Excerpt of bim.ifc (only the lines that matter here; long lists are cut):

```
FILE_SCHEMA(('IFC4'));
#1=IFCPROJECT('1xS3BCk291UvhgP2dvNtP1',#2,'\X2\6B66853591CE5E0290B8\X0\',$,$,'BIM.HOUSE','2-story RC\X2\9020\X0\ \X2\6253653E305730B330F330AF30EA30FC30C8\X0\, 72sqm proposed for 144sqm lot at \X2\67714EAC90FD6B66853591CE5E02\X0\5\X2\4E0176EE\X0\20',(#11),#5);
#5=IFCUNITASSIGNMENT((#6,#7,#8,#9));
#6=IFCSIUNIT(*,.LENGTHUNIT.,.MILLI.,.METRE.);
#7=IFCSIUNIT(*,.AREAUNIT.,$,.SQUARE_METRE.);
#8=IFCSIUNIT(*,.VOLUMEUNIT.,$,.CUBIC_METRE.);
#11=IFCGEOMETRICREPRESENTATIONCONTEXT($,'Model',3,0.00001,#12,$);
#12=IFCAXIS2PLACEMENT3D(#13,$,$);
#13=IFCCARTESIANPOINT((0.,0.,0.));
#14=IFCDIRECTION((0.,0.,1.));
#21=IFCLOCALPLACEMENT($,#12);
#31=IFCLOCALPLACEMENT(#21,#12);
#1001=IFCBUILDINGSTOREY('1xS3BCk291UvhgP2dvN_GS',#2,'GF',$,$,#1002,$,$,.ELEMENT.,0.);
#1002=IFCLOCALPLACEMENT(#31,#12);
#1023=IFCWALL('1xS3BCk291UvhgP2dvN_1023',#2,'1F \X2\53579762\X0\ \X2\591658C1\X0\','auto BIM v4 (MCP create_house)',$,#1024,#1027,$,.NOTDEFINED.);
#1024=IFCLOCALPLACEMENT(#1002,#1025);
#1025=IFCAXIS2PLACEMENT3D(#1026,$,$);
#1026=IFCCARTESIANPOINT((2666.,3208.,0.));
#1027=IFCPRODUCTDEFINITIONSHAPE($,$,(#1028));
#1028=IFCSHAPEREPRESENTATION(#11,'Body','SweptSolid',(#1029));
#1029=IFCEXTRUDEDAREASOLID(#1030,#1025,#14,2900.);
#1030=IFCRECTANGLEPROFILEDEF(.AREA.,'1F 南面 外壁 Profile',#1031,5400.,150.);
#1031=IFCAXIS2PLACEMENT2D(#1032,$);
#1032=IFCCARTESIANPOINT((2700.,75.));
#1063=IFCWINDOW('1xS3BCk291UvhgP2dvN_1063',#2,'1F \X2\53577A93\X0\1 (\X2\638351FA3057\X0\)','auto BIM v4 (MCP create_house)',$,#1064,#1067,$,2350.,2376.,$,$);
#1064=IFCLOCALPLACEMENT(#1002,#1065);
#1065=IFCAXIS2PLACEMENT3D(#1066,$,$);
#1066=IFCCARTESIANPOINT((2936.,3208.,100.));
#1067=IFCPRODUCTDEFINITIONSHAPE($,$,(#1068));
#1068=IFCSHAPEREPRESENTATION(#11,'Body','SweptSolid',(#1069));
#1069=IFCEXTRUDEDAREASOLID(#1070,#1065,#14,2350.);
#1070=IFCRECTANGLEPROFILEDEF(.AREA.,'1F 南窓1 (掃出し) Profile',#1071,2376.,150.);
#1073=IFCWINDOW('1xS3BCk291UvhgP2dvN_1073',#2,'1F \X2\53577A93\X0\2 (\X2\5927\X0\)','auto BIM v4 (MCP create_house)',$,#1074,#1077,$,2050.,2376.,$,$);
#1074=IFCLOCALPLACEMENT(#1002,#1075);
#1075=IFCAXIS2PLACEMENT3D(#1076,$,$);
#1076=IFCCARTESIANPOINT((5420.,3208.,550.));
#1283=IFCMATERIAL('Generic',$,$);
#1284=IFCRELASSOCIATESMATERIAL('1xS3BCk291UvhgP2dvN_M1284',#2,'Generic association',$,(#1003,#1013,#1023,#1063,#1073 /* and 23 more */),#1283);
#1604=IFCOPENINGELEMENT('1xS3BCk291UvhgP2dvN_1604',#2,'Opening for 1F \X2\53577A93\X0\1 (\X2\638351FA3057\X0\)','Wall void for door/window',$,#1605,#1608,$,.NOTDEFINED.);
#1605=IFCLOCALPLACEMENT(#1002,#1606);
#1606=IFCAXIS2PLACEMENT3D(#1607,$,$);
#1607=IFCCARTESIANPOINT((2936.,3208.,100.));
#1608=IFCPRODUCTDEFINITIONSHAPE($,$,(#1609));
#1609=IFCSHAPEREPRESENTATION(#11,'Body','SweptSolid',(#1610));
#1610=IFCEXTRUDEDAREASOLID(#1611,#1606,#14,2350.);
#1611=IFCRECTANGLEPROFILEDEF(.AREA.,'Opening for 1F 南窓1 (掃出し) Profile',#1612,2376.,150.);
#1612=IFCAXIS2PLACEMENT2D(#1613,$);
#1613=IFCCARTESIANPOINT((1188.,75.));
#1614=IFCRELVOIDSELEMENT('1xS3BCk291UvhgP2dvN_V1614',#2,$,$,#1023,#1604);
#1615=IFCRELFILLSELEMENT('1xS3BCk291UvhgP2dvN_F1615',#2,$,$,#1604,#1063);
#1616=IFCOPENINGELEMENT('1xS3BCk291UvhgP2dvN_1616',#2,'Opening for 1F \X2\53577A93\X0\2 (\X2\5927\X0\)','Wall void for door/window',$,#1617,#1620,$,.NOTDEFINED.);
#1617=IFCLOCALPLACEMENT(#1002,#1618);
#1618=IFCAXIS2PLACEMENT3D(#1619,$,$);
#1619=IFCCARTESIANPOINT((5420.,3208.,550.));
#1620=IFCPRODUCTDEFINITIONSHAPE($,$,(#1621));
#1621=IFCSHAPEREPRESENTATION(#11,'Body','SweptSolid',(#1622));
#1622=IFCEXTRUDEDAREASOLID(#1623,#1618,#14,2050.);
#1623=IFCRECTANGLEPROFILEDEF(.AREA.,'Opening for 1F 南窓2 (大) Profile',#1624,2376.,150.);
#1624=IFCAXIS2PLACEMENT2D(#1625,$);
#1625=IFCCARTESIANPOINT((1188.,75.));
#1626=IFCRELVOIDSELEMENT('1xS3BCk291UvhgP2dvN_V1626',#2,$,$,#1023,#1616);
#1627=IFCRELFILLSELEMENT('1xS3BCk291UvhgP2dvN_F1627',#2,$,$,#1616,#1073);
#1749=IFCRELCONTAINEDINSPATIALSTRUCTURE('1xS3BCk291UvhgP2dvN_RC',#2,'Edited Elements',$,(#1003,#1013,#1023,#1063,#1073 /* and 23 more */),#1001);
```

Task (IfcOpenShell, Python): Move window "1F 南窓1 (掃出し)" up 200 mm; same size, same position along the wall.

```python
import numpy as np
import ifcopenshell
import ifcopenshell.api.geometry
import ifcopenshell.util.placement
import ifcopenshell.util.unit

model = ifcopenshell.open("bim.ifc")
unit_scale = ifcopenshell.util.unit.calculate_unit_scale(model)

window = model.by_guid("1xS3BCk291UvhgP2dvN_1063")
opening = window.FillsVoids[0].RelatingOpeningElement
dz = 0.2 / unit_scale

shift = np.array([0.0, 0.0, dz])
# The window is not placed relative to its opening, so move both.
for product in (opening, window):
    matrix = ifcopenshell.util.placement.get_local_placement(product.ObjectPlacement)
    matrix[:3, 3] += shift
    ifcopenshell.api.geometry.edit_object_placement(model, product=product, matrix=matrix, is_si=False)

print(f"moved by {dz * unit_scale:+.3f} m")

model.write("bim_edited.ifc")
```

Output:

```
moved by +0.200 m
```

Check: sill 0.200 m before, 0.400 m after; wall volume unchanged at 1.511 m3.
